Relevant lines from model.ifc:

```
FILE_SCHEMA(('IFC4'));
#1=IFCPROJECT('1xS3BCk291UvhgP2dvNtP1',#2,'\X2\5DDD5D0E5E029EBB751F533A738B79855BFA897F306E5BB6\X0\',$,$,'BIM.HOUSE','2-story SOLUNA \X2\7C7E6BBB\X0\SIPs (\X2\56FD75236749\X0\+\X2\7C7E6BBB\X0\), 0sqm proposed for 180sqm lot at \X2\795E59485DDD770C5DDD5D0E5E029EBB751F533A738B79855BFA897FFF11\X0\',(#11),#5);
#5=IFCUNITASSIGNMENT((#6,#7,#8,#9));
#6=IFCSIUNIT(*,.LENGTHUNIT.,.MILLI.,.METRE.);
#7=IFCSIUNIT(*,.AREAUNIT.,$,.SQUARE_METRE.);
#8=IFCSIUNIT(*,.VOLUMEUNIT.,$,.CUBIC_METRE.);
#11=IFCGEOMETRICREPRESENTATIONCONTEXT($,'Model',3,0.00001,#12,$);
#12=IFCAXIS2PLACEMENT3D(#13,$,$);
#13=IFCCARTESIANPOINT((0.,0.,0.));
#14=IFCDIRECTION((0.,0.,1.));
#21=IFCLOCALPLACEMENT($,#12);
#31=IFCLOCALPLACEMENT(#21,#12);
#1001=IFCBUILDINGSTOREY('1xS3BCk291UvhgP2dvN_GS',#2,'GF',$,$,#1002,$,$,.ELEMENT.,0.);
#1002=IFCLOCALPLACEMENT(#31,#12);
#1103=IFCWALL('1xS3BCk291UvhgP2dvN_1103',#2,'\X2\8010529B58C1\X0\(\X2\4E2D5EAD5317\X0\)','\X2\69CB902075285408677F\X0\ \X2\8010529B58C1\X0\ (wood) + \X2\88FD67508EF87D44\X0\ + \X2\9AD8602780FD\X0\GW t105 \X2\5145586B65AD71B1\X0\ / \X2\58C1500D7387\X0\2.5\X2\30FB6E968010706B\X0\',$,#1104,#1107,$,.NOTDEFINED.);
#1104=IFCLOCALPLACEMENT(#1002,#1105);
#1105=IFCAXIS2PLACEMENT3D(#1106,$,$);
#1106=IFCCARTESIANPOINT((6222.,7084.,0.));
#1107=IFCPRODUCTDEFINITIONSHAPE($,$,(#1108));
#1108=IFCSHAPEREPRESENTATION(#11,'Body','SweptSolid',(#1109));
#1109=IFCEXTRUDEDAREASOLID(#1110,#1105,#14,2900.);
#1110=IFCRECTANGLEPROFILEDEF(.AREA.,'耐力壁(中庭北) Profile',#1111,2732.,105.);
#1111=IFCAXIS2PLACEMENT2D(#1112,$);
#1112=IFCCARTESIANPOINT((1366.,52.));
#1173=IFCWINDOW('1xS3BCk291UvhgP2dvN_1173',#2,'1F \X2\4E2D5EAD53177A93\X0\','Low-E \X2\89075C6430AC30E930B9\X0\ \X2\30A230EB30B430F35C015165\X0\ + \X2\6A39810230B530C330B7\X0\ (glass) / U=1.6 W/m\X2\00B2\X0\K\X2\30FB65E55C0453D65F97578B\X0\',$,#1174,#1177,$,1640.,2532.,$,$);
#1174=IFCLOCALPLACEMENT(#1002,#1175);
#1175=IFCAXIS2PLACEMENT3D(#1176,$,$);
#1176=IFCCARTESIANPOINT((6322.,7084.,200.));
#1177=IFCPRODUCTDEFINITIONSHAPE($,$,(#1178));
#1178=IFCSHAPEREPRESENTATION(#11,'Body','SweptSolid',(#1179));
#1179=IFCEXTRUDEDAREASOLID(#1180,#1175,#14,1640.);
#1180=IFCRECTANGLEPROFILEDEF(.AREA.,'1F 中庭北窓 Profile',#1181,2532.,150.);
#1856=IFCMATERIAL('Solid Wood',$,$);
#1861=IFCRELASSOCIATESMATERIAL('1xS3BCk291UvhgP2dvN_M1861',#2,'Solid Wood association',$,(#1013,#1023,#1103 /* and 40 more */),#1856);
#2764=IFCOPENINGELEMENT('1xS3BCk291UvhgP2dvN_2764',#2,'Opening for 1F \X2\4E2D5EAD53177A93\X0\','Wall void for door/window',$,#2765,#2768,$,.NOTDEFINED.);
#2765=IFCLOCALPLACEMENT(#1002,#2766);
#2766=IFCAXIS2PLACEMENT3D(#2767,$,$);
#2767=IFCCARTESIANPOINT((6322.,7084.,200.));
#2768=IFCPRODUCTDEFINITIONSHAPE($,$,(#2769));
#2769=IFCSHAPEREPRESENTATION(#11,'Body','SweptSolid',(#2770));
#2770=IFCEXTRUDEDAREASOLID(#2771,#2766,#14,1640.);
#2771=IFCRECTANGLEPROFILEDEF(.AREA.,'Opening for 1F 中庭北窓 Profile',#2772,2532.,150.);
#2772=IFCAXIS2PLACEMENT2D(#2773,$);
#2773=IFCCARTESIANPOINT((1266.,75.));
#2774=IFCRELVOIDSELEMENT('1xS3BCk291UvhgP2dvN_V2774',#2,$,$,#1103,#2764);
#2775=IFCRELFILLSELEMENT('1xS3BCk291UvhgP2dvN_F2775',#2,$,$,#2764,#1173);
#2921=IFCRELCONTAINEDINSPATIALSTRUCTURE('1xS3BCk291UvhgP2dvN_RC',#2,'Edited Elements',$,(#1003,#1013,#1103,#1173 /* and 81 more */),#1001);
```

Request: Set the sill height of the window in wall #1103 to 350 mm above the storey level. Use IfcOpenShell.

```python
import numpy as np
import ifcopenshell
import ifcopenshell.api.geometry
import ifcopenshell.geom
import ifcopenshell.util.element
import ifcopenshell.util.placement
import ifcopenshell.util.shape
import ifcopenshell.util.unit

model = ifcopenshell.open("model.ifc")
unit_scale = ifcopenshell.util.unit.calculate_unit_scale(model)

window = model.by_guid("1xS3BCk291UvhgP2dvN_1173")
opening = window.FillsVoids[0].RelatingOpeningElement
storey = ifcopenshell.util.element.get_container(window, ifc_class="IfcBuildingStorey")
level = ifcopenshell.util.placement.get_local_placement(storey.ObjectPlacement)[2, 3]

# The opening's origin need not be at the sill, so measure its lowest point.
shape = ifcopenshell.geom.create_shape(ifcopenshell.geom.settings(), opening)
bottom = ifcopenshell.util.shape.get_shape_bottom_elevation(shape, shape.geometry) / unit_scale
dz = level + 0.35 / unit_scale - bottom

shift = np.array([0.0, 0.0, dz])
# The window is not placed relative to its opening, so move both.
for product in (opening, window):
    matrix = ifcopenshell.util.placement.get_local_placement(product.ObjectPlacement)
    matrix[:3, 3] += shift
    ifcopenshell.api.geometry.edit_object_placement(model, product=product, matrix=matrix, is_si=False)

print(f"moved by {dz * unit_scale:+.3f} m")

model.write("model_v2.ifc")
```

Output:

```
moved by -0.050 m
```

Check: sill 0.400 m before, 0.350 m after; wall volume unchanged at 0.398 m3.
